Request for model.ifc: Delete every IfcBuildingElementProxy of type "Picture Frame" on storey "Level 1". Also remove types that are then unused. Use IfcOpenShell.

First a look at what the model holds.

```python
import ifcopenshell
import ifcopenshell.util.element

model = ifcopenshell.open("model.ifc")
print(model.schema)
storey = next(s for s in model.by_type("IfcBuildingStorey") if s.Name == "Level 1")
proxies = [e for e in ifcopenshell.util.element.get_decomposition(storey) if e.is_a("IfcBuildingElementProxy")]
seen = {}
for e in proxies:
    element_type = ifcopenshell.util.element.get_type(e)
    name = element_type.Name if element_type not in (None, e) else None
    seen[name] = seen.get(name, 0) + 1
for name, count in sorted(seen.items(), key=str):
    print(count, "x", name)
```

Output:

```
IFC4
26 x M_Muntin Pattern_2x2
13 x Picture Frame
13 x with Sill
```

```python
import ifcopenshell
import ifcopenshell.api.root
import ifcopenshell.util.element

model = ifcopenshell.open("model.ifc")

storey = next(s for s in model.by_type("IfcBuildingStorey") if s.Name == "Level 1")
proxies = [e for e in ifcopenshell.util.element.get_decomposition(storey) if e.is_a("IfcBuildingElementProxy")]
targets = [e for e in proxies if (t := ifcopenshell.util.element.get_type(e)) not in (None, e) and t.Name == "Picture Frame"]
types = {ifcopenshell.util.element.get_type(e) for e in targets} - {None, *targets}

for e in targets:
    ifcopenshell.api.root.remove_product(model, product=e)
print(len(targets), "removed")

unused = [t for t in types if not ifcopenshell.util.element.get_types(t)]
for t in unused:
    ifcopenshell.api.root.remove_product(model, product=t)
print(len(unused), "unused types removed")

model.write("model_updated.ifc")
```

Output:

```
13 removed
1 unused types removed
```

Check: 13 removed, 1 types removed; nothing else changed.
